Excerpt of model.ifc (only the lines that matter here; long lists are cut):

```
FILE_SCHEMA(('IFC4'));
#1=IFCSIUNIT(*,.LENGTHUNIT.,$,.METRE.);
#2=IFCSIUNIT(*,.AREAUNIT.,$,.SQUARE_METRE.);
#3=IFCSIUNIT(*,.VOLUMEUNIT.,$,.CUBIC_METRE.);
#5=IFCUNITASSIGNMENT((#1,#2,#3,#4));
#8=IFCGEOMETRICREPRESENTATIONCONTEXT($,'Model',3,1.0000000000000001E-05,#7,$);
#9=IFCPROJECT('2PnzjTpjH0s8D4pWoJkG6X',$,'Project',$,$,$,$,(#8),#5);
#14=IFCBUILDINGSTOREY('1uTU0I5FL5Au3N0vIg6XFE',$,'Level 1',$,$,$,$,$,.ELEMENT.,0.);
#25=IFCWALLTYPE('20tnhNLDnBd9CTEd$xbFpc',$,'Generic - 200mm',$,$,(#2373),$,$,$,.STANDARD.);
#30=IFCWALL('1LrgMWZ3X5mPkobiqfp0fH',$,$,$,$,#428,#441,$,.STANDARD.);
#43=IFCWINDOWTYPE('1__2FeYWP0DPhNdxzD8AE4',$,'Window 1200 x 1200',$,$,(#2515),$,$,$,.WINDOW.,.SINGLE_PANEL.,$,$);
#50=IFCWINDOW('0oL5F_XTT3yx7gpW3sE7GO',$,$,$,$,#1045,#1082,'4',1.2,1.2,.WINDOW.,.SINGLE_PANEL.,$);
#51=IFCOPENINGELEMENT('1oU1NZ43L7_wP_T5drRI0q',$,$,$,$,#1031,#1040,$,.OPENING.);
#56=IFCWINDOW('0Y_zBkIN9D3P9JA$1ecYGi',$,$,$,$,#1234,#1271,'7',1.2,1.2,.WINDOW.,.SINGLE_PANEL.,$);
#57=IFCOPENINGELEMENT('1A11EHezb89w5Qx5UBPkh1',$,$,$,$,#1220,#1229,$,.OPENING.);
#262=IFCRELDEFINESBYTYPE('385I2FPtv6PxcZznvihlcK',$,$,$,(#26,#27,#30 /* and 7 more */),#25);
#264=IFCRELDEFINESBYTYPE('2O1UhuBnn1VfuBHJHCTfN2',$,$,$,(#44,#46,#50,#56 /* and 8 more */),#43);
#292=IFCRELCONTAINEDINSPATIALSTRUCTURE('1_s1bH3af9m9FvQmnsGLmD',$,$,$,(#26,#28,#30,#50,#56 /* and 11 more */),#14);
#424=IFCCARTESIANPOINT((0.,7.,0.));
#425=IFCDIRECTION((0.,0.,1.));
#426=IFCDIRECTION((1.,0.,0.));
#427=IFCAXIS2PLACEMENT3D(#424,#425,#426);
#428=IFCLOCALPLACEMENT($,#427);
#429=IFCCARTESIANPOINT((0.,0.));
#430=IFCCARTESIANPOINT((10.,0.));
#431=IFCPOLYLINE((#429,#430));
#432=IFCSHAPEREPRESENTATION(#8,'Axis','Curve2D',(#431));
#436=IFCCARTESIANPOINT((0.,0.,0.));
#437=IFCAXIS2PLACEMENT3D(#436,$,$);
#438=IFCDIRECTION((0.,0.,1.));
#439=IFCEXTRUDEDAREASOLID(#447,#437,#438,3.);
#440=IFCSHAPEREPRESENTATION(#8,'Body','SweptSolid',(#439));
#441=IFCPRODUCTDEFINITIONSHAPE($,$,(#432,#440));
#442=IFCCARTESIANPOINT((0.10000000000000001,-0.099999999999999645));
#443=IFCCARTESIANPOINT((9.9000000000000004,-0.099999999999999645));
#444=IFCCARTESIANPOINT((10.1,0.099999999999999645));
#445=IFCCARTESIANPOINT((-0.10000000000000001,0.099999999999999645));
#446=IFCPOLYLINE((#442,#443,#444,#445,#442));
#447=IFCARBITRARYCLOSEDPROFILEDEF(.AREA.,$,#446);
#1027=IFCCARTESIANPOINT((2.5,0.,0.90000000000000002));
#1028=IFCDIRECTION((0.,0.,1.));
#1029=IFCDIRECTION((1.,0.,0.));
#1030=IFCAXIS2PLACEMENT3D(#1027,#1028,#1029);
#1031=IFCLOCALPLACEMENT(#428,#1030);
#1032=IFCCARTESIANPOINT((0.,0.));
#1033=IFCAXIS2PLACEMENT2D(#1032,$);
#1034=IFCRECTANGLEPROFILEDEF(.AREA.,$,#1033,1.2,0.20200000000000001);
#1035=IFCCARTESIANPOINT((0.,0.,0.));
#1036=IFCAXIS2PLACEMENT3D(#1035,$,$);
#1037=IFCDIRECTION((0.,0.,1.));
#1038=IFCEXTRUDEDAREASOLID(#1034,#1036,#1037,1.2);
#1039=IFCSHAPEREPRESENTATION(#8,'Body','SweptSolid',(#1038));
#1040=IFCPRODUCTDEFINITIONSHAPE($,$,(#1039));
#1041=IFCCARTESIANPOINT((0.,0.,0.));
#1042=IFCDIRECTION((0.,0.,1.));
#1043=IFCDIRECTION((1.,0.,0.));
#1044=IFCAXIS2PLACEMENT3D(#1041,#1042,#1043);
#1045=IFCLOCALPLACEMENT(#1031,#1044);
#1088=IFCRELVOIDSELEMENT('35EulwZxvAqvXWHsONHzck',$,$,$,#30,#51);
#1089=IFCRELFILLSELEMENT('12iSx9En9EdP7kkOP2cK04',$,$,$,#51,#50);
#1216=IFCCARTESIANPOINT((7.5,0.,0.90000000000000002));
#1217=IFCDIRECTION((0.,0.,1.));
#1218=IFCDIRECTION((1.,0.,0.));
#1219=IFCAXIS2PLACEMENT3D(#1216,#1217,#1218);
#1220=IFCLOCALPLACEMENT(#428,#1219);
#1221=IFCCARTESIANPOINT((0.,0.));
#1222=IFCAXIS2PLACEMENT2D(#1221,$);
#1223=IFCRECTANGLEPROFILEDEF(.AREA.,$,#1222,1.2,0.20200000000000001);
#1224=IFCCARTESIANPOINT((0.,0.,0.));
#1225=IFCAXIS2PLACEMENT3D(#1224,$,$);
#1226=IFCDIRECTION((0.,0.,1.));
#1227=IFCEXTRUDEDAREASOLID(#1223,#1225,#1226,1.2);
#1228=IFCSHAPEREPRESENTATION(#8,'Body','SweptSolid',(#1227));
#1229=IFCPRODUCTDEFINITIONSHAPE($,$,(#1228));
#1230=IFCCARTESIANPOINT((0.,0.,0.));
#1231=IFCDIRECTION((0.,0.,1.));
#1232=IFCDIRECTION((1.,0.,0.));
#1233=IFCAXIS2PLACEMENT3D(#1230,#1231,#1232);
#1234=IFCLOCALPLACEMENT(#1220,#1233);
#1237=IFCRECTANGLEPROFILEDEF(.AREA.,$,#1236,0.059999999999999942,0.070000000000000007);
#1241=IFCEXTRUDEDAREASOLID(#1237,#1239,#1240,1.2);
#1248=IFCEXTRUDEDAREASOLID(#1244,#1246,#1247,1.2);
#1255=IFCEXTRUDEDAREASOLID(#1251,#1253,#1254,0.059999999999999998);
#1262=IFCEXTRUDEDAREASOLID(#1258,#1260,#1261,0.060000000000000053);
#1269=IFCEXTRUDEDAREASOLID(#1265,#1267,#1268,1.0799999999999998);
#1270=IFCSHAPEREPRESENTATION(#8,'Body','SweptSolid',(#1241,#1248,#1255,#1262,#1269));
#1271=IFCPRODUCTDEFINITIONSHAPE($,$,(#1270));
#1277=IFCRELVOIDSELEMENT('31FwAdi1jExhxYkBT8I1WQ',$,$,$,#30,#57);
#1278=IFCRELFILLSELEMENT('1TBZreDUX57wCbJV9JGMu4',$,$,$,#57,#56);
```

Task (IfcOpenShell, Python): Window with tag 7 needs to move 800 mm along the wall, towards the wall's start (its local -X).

```python
import ifcopenshell
import ifcopenshell.api.geometry
import ifcopenshell.util.placement
import ifcopenshell.util.unit

model = ifcopenshell.open("model.ifc")
unit_scale = ifcopenshell.util.unit.calculate_unit_scale(model)

window = model.by_guid("0Y_zBkIN9D3P9JA$1ecYGi")
opening = window.FillsVoids[0].RelatingOpeningElement
wall = opening.VoidsElements[0].RelatingBuildingElement

wall_matrix = ifcopenshell.util.placement.get_local_placement(wall.ObjectPlacement)
shift = wall_matrix[:3, 0] * -0.8 / unit_scale
before = ifcopenshell.util.placement.get_local_placement(window.ObjectPlacement)[:3, 3].copy()

# The window is placed relative to its opening, so it follows when the opening moves.
matrix = ifcopenshell.util.placement.get_local_placement(opening.ObjectPlacement)
matrix[:3, 3] += shift
ifcopenshell.api.geometry.edit_object_placement(
    model, product=opening, matrix=matrix, is_si=False, should_transform_children=True
)

after = ifcopenshell.util.placement.get_local_placement(window.ObjectPlacement)[:3, 3]
print("window moved by", (after - before).round(3) + 0.0)

model.write("model_edited.ifc")
```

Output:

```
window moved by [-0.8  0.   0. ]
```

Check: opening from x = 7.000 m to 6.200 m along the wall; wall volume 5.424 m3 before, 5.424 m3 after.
